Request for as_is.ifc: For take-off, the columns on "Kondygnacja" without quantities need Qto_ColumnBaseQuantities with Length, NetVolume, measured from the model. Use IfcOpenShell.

First a look at what the model holds.

```python
import ifcopenshell
import ifcopenshell.util.element
import ifcopenshell.util.unit

model = ifcopenshell.open("as_is.ifc")
print(model.schema)
for unit_type in ("LENGTHUNIT", "AREAUNIT", "VOLUMEUNIT"):
    print(unit_type, ifcopenshell.util.unit.calculate_unit_scale(model, unit_type))
storey = next(s for s in model.by_type("IfcBuildingStorey") if s.Name == "Kondygnacja")
columns = [e for e in ifcopenshell.util.element.get_decomposition(storey) if e.is_a("IfcColumn")]
for e in sorted(columns, key=lambda e: e.id()):
    print(e.id(), e.is_a(), e.Name, list(ifcopenshell.util.element.get_psets(e, qtos_only=True)), sep=" | ")
```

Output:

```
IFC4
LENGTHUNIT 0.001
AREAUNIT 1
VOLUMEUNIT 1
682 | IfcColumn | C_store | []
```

```python
import ifcopenshell
import ifcopenshell.api.pset
import ifcopenshell.geom
import ifcopenshell.util.element
import ifcopenshell.util.shape
import ifcopenshell.util.unit

model = ifcopenshell.open("as_is.ifc")
unit_scale = ifcopenshell.util.unit.calculate_unit_scale(model)
volume_scale = ifcopenshell.util.unit.calculate_unit_scale(model, "VOLUMEUNIT")
settings = ifcopenshell.geom.settings()

storey = next(s for s in model.by_type("IfcBuildingStorey") if s.Name == "Kondygnacja")
columns = [e for e in ifcopenshell.util.element.get_decomposition(storey) if e.is_a("IfcColumn")]

for e in sorted(columns, key=lambda e: e.id()):
    if ifcopenshell.util.element.get_psets(e, qtos_only=True, should_inherit=False):
        continue
    # Geometry comes back in metres, in the element's own axes.
    shape = ifcopenshell.geom.create_shape(settings, e)
    values = {
        "Length": ifcopenshell.util.shape.get_z(shape.geometry) / unit_scale,
        "NetVolume": ifcopenshell.util.shape.get_volume(shape.geometry) / volume_scale,
    }
    qto = ifcopenshell.api.pset.add_qto(model, product=e, name="Qto_ColumnBaseQuantities")
    ifcopenshell.api.pset.edit_qto(model, qto=qto, properties=values)
    print(e.id(), {k: round(v, 3) for k, v in values.items()})

model.write("as_is_v2.ifc")
```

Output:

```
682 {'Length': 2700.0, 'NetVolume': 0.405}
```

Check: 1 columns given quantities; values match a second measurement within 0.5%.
